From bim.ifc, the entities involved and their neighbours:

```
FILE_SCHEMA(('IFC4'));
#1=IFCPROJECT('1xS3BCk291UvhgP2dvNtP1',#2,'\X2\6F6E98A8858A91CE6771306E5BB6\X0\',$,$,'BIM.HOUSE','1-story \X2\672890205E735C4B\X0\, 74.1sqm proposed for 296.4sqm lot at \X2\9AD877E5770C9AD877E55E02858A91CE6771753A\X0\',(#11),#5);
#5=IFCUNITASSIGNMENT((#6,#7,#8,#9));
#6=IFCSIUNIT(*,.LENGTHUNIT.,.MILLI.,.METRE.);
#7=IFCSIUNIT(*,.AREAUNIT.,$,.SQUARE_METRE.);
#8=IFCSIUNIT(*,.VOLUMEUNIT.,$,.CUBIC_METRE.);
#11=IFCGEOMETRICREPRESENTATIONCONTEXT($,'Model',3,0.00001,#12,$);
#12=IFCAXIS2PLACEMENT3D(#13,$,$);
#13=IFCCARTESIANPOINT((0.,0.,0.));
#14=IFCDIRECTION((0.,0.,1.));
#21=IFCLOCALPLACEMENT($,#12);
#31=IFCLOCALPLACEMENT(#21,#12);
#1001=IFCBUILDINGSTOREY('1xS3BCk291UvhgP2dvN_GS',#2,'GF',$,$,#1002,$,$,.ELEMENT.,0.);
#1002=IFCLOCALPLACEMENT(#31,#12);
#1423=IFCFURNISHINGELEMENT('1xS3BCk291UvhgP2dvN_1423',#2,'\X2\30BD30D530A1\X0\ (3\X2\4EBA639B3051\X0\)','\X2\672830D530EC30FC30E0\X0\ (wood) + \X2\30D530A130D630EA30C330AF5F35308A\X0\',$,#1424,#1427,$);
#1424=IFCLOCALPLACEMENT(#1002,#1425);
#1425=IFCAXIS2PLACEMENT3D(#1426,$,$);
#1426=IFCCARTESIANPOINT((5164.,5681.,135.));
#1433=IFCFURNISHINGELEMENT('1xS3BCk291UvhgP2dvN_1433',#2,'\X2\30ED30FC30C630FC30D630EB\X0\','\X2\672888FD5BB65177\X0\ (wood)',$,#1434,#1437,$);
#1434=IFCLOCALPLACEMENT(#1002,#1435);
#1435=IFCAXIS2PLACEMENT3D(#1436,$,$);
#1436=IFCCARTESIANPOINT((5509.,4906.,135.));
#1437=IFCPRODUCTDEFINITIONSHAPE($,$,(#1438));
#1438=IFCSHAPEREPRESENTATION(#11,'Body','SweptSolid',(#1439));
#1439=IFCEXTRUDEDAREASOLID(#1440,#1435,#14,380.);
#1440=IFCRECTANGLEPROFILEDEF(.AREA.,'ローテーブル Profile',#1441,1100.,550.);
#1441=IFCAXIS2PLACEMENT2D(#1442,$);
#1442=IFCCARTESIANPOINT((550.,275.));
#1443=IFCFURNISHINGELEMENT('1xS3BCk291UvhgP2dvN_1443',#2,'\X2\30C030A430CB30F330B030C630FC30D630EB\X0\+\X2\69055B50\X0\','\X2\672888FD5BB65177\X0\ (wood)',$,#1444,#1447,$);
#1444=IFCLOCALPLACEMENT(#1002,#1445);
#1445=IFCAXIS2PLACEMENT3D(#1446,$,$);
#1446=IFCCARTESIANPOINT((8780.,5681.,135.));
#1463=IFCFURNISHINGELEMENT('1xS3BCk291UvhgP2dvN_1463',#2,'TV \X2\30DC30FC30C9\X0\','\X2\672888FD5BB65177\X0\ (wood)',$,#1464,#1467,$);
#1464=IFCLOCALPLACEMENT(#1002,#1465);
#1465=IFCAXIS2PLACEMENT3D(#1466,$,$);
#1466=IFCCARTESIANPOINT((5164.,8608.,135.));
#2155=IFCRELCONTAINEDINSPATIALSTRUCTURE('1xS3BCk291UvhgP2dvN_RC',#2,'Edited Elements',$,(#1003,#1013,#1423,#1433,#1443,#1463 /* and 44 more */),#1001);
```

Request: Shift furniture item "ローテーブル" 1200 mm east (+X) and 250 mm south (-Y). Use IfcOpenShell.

```python
import ifcopenshell
import ifcopenshell.api.geometry
import ifcopenshell.util.placement
import ifcopenshell.util.unit

model = ifcopenshell.open("bim.ifc")
unit_scale = ifcopenshell.util.unit.calculate_unit_scale(model)

item = model.by_guid("1xS3BCk291UvhgP2dvN_1433")
matrix = ifcopenshell.util.placement.get_local_placement(item.ObjectPlacement)
matrix[0, 3] += 1.2 / unit_scale
matrix[1, 3] -= 0.25 / unit_scale
ifcopenshell.api.geometry.edit_object_placement(model, product=item, matrix=matrix, is_si=False)

print(ifcopenshell.util.placement.get_local_placement(item.ObjectPlacement).round(3) + 0.0)

model.write("bim_rev.ifc")
```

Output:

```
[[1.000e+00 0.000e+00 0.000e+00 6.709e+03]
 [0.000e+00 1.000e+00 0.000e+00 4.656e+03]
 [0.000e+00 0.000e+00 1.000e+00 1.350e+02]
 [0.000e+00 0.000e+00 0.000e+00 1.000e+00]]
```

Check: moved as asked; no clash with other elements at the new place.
